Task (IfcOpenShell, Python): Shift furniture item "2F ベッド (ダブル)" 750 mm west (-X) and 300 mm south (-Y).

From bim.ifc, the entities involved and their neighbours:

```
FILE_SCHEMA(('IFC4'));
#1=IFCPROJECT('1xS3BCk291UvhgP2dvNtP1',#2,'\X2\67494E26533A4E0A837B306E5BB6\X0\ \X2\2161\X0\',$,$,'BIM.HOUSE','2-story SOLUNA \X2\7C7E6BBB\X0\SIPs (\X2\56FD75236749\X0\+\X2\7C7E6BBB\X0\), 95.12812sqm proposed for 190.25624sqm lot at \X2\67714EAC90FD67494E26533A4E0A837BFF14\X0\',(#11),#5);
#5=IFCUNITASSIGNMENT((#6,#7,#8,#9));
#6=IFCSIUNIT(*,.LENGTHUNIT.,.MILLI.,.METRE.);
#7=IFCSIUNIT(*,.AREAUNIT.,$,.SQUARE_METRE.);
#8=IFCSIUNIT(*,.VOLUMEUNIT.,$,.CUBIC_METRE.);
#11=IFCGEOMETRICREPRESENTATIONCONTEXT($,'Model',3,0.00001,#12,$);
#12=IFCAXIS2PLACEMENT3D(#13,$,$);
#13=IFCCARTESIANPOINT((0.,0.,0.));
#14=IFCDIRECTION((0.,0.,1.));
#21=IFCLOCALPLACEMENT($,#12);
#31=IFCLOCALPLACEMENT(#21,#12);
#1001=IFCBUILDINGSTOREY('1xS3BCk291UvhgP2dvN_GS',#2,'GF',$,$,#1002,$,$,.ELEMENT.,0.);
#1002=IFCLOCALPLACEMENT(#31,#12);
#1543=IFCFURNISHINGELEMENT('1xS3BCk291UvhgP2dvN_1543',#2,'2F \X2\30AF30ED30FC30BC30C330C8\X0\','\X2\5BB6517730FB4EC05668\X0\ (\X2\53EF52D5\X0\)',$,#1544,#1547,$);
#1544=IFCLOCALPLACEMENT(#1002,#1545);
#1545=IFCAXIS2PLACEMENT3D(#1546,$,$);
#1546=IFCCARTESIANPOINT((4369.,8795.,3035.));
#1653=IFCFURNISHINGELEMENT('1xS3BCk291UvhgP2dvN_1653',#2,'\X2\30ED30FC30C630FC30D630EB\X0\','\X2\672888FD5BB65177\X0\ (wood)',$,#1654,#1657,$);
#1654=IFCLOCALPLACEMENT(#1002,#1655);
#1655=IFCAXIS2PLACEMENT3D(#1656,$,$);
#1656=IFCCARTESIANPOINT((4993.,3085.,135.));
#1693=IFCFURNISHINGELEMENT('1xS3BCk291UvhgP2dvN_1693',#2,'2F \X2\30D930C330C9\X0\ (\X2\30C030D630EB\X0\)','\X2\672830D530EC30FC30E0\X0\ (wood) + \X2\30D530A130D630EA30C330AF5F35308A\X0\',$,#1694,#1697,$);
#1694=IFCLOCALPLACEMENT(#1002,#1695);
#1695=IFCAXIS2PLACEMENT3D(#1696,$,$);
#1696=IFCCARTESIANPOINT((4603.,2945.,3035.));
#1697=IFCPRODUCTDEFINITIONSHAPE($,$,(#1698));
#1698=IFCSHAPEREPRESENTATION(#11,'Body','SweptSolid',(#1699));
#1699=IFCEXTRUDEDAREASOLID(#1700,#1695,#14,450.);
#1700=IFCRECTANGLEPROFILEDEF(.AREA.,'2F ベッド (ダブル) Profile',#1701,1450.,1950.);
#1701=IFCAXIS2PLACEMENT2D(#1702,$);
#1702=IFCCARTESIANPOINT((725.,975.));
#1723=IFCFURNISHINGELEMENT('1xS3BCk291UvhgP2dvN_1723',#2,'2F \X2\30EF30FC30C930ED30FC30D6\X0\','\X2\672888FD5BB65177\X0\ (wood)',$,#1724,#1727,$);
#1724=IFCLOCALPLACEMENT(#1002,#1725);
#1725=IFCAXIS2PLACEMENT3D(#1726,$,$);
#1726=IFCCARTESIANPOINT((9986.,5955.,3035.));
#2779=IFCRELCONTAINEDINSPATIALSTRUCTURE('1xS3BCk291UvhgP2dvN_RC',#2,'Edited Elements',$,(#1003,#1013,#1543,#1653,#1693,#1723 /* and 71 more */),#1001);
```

```python
import ifcopenshell
import ifcopenshell.api.geometry
import ifcopenshell.util.placement
import ifcopenshell.util.unit

model = ifcopenshell.open("bim.ifc")
unit_scale = ifcopenshell.util.unit.calculate_unit_scale(model)

item = model.by_id(1693)
matrix = ifcopenshell.util.placement.get_local_placement(item.ObjectPlacement)
matrix[0, 3] -= 0.75 / unit_scale
matrix[1, 3] -= 0.3 / unit_scale
ifcopenshell.api.geometry.edit_object_placement(model, product=item, matrix=matrix, is_si=False)

print(ifcopenshell.util.placement.get_local_placement(item.ObjectPlacement).round(3) + 0.0)

model.write("bim_v2.ifc")
```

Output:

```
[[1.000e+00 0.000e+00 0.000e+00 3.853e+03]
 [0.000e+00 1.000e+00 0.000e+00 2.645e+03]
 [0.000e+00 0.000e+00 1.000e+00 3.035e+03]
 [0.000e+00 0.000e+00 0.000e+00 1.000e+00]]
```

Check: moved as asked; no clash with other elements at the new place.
